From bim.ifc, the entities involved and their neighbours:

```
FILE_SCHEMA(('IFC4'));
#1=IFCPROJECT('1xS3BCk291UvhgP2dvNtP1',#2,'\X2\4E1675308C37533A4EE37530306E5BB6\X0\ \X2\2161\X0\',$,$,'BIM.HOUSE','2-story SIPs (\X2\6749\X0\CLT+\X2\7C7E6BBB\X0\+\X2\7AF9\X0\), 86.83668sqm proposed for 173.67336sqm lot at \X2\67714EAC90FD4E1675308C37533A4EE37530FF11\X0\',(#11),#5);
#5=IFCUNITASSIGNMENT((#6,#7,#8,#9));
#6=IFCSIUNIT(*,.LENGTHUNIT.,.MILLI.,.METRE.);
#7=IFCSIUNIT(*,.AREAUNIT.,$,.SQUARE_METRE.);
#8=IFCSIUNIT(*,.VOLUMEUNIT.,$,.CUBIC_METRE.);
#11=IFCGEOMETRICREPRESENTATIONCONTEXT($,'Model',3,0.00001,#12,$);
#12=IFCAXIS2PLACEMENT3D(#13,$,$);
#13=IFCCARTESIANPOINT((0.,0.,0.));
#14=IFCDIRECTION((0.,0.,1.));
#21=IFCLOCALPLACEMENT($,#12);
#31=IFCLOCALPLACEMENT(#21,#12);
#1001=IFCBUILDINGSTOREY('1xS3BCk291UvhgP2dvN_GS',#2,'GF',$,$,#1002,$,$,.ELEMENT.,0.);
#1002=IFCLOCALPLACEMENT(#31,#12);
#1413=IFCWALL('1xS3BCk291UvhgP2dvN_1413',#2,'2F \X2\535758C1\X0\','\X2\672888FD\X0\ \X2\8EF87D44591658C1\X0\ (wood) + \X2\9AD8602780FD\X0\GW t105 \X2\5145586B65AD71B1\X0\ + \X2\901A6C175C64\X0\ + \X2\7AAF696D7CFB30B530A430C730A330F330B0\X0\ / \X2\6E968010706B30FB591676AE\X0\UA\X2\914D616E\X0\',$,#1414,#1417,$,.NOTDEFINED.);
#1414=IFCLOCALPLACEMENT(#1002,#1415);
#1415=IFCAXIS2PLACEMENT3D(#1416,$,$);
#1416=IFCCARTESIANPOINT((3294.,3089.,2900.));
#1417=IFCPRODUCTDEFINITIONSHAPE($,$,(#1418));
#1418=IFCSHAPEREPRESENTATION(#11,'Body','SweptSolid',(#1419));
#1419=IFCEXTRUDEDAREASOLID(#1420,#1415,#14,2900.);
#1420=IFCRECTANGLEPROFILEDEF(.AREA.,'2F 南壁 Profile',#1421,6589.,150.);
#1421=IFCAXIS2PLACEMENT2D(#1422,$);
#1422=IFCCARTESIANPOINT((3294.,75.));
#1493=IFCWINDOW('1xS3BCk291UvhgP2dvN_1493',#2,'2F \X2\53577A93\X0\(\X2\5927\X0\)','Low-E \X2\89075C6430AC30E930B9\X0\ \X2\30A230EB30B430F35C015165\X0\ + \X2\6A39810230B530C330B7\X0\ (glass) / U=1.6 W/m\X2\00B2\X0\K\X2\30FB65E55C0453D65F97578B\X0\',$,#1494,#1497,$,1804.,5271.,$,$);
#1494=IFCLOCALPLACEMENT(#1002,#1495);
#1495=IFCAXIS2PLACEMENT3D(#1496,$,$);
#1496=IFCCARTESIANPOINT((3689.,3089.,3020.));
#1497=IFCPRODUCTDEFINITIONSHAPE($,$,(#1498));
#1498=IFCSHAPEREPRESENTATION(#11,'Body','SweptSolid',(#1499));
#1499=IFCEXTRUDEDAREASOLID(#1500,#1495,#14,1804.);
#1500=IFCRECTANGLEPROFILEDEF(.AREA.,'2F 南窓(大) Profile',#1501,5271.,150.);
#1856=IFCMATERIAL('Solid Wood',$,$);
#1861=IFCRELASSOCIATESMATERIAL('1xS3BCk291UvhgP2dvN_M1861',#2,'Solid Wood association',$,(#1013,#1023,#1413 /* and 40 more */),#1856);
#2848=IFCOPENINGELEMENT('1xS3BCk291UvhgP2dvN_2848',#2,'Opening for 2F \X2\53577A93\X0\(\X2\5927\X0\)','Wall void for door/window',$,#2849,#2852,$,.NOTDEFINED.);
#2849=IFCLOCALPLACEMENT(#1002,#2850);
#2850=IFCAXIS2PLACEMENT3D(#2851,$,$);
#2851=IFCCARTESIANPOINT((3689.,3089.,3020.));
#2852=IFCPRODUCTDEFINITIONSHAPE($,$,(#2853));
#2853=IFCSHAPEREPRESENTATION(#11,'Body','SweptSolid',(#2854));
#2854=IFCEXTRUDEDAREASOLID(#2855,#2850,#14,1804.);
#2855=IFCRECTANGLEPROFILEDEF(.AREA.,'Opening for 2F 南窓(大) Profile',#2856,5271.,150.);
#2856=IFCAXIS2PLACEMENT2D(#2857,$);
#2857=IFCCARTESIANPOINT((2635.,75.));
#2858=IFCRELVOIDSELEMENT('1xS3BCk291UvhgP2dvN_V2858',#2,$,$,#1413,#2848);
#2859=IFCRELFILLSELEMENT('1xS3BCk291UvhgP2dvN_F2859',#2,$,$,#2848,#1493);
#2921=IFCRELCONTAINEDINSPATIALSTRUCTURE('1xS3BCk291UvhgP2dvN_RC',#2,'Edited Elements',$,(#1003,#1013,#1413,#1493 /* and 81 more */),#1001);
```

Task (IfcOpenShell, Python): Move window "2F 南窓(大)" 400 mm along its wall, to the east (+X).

```python
import ifcopenshell
import ifcopenshell.api.geometry
import ifcopenshell.util.placement

model = ifcopenshell.open("bim.ifc")

window = model.by_guid("1xS3BCk291UvhgP2dvN_1493")
opening = window.FillsVoids[0].RelatingOpeningElement
wall = opening.VoidsElements[0].RelatingBuildingElement

wall_matrix = ifcopenshell.util.placement.get_local_placement(wall.ObjectPlacement)
shift = wall_matrix[:3, 0] * 400.0
before = ifcopenshell.util.placement.get_local_placement(window.ObjectPlacement)[:3, 3].copy()

# The window is not placed relative to its opening, so move both.
for product in (opening, window):
    matrix = ifcopenshell.util.placement.get_local_placement(product.ObjectPlacement)
    matrix[:3, 3] += shift
    ifcopenshell.api.geometry.edit_object_placement(model, product=product, matrix=matrix, is_si=False)

after = ifcopenshell.util.placement.get_local_placement(window.ObjectPlacement)[:3, 3]
print("window moved by", (after - before).round(3) + 0.0)

model.write("bim_v2.ifc")
```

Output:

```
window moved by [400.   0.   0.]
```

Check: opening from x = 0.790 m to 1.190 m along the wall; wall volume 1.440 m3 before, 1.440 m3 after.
